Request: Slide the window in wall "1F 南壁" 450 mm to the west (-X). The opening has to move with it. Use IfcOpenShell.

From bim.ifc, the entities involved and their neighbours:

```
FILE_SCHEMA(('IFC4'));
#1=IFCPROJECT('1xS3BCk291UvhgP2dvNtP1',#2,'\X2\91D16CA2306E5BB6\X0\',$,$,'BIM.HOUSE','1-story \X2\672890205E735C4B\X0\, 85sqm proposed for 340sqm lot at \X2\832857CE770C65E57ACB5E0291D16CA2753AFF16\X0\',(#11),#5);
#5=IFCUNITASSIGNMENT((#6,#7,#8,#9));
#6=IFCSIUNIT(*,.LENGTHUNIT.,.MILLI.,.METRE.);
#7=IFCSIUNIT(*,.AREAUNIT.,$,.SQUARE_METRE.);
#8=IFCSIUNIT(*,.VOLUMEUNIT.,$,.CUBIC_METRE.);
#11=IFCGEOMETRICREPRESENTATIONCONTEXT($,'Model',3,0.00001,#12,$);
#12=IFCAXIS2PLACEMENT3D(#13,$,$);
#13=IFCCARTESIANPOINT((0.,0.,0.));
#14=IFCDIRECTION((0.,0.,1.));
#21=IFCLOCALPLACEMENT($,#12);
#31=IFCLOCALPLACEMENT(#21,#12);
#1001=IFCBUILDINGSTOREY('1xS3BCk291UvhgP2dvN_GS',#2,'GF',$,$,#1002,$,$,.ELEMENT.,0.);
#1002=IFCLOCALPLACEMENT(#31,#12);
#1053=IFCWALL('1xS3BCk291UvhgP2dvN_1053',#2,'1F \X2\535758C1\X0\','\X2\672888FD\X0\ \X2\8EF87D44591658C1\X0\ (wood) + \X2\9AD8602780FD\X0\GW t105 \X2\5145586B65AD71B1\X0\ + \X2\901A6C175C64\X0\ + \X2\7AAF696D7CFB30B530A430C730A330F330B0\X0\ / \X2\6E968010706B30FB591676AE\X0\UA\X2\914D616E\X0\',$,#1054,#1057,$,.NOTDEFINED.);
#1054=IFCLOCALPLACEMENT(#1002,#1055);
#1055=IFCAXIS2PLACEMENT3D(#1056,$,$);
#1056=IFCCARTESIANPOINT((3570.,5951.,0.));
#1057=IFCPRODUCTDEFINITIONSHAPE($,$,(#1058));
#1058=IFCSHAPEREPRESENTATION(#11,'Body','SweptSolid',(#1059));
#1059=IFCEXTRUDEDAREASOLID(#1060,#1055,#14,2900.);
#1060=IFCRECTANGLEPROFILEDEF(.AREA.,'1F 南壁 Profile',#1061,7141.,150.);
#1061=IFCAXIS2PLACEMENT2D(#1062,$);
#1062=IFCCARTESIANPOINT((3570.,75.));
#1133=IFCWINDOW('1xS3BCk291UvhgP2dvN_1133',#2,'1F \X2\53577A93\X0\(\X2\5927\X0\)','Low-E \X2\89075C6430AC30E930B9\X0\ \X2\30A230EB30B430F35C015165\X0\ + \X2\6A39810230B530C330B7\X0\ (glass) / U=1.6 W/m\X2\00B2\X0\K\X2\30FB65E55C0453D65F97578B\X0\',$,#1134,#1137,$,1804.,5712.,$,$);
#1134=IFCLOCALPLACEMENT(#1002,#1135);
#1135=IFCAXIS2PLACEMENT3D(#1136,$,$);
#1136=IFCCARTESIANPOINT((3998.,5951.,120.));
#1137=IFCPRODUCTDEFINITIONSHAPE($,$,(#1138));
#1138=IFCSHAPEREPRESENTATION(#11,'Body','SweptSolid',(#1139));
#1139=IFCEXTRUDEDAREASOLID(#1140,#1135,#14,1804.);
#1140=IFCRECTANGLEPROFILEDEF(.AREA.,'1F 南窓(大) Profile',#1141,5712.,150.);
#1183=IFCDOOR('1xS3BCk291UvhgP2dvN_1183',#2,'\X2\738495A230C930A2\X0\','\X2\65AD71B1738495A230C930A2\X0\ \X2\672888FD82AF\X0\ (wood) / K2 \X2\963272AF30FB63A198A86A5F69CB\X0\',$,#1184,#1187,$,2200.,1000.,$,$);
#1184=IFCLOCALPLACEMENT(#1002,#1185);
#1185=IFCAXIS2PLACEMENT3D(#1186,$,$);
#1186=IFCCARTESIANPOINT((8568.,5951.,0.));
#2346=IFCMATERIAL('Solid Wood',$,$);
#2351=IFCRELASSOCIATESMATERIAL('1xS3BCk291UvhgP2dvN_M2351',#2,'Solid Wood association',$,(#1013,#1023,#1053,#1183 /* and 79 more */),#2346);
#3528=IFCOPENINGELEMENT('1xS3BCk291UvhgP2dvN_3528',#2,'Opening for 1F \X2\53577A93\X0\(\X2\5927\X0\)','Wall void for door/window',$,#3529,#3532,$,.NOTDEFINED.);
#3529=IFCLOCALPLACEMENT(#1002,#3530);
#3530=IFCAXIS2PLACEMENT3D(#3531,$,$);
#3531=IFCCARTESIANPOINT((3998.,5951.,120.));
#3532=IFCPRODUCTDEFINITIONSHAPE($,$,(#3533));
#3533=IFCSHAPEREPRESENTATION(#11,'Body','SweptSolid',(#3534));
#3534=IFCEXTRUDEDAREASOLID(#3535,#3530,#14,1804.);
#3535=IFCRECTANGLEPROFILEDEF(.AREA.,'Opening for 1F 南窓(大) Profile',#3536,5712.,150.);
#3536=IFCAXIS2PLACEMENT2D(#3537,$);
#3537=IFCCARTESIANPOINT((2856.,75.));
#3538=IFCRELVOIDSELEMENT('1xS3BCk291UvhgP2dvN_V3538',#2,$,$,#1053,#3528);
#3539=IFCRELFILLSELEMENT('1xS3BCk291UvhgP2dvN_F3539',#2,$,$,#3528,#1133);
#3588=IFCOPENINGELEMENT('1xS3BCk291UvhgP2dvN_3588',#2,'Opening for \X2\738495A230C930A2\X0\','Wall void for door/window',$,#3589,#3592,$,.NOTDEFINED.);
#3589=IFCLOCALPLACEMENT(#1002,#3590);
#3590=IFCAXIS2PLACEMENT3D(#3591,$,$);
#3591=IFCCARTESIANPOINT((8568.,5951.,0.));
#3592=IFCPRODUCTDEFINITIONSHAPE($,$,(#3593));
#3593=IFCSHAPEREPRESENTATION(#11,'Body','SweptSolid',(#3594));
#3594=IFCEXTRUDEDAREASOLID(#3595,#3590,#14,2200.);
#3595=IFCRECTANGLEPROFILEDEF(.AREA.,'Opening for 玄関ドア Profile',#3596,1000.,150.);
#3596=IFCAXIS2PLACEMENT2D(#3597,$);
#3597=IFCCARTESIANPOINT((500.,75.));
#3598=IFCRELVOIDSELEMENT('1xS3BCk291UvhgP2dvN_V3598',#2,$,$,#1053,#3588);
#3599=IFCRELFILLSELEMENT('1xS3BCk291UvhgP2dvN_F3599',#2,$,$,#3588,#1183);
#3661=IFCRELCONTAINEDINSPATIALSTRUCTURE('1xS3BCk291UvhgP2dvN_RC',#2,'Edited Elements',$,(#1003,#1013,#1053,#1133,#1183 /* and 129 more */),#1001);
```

```python
import ifcopenshell
import ifcopenshell.api.geometry
import ifcopenshell.util.placement
import ifcopenshell.util.unit

model = ifcopenshell.open("bim.ifc")
unit_scale = ifcopenshell.util.unit.calculate_unit_scale(model)

window = model.by_id(1133)
opening = window.FillsVoids[0].RelatingOpeningElement
wall = opening.VoidsElements[0].RelatingBuildingElement

wall_matrix = ifcopenshell.util.placement.get_local_placement(wall.ObjectPlacement)
shift = wall_matrix[:3, 0] * -0.45 / unit_scale
before = ifcopenshell.util.placement.get_local_placement(window.ObjectPlacement)[:3, 3].copy()

# The window is not placed relative to its opening, so move both.
for product in (opening, window):
    matrix = ifcopenshell.util.placement.get_local_placement(product.ObjectPlacement)
    matrix[:3, 3] += shift
    ifcopenshell.api.geometry.edit_object_placement(model, product=product, matrix=matrix, is_si=False)

after = ifcopenshell.util.placement.get_local_placement(window.ObjectPlacement)[:3, 3]
print("window moved by", (after - before).round(3) + 0.0)

model.write("bim_v2.ifc")
```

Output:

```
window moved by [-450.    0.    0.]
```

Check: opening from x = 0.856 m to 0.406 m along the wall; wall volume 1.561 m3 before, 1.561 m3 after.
